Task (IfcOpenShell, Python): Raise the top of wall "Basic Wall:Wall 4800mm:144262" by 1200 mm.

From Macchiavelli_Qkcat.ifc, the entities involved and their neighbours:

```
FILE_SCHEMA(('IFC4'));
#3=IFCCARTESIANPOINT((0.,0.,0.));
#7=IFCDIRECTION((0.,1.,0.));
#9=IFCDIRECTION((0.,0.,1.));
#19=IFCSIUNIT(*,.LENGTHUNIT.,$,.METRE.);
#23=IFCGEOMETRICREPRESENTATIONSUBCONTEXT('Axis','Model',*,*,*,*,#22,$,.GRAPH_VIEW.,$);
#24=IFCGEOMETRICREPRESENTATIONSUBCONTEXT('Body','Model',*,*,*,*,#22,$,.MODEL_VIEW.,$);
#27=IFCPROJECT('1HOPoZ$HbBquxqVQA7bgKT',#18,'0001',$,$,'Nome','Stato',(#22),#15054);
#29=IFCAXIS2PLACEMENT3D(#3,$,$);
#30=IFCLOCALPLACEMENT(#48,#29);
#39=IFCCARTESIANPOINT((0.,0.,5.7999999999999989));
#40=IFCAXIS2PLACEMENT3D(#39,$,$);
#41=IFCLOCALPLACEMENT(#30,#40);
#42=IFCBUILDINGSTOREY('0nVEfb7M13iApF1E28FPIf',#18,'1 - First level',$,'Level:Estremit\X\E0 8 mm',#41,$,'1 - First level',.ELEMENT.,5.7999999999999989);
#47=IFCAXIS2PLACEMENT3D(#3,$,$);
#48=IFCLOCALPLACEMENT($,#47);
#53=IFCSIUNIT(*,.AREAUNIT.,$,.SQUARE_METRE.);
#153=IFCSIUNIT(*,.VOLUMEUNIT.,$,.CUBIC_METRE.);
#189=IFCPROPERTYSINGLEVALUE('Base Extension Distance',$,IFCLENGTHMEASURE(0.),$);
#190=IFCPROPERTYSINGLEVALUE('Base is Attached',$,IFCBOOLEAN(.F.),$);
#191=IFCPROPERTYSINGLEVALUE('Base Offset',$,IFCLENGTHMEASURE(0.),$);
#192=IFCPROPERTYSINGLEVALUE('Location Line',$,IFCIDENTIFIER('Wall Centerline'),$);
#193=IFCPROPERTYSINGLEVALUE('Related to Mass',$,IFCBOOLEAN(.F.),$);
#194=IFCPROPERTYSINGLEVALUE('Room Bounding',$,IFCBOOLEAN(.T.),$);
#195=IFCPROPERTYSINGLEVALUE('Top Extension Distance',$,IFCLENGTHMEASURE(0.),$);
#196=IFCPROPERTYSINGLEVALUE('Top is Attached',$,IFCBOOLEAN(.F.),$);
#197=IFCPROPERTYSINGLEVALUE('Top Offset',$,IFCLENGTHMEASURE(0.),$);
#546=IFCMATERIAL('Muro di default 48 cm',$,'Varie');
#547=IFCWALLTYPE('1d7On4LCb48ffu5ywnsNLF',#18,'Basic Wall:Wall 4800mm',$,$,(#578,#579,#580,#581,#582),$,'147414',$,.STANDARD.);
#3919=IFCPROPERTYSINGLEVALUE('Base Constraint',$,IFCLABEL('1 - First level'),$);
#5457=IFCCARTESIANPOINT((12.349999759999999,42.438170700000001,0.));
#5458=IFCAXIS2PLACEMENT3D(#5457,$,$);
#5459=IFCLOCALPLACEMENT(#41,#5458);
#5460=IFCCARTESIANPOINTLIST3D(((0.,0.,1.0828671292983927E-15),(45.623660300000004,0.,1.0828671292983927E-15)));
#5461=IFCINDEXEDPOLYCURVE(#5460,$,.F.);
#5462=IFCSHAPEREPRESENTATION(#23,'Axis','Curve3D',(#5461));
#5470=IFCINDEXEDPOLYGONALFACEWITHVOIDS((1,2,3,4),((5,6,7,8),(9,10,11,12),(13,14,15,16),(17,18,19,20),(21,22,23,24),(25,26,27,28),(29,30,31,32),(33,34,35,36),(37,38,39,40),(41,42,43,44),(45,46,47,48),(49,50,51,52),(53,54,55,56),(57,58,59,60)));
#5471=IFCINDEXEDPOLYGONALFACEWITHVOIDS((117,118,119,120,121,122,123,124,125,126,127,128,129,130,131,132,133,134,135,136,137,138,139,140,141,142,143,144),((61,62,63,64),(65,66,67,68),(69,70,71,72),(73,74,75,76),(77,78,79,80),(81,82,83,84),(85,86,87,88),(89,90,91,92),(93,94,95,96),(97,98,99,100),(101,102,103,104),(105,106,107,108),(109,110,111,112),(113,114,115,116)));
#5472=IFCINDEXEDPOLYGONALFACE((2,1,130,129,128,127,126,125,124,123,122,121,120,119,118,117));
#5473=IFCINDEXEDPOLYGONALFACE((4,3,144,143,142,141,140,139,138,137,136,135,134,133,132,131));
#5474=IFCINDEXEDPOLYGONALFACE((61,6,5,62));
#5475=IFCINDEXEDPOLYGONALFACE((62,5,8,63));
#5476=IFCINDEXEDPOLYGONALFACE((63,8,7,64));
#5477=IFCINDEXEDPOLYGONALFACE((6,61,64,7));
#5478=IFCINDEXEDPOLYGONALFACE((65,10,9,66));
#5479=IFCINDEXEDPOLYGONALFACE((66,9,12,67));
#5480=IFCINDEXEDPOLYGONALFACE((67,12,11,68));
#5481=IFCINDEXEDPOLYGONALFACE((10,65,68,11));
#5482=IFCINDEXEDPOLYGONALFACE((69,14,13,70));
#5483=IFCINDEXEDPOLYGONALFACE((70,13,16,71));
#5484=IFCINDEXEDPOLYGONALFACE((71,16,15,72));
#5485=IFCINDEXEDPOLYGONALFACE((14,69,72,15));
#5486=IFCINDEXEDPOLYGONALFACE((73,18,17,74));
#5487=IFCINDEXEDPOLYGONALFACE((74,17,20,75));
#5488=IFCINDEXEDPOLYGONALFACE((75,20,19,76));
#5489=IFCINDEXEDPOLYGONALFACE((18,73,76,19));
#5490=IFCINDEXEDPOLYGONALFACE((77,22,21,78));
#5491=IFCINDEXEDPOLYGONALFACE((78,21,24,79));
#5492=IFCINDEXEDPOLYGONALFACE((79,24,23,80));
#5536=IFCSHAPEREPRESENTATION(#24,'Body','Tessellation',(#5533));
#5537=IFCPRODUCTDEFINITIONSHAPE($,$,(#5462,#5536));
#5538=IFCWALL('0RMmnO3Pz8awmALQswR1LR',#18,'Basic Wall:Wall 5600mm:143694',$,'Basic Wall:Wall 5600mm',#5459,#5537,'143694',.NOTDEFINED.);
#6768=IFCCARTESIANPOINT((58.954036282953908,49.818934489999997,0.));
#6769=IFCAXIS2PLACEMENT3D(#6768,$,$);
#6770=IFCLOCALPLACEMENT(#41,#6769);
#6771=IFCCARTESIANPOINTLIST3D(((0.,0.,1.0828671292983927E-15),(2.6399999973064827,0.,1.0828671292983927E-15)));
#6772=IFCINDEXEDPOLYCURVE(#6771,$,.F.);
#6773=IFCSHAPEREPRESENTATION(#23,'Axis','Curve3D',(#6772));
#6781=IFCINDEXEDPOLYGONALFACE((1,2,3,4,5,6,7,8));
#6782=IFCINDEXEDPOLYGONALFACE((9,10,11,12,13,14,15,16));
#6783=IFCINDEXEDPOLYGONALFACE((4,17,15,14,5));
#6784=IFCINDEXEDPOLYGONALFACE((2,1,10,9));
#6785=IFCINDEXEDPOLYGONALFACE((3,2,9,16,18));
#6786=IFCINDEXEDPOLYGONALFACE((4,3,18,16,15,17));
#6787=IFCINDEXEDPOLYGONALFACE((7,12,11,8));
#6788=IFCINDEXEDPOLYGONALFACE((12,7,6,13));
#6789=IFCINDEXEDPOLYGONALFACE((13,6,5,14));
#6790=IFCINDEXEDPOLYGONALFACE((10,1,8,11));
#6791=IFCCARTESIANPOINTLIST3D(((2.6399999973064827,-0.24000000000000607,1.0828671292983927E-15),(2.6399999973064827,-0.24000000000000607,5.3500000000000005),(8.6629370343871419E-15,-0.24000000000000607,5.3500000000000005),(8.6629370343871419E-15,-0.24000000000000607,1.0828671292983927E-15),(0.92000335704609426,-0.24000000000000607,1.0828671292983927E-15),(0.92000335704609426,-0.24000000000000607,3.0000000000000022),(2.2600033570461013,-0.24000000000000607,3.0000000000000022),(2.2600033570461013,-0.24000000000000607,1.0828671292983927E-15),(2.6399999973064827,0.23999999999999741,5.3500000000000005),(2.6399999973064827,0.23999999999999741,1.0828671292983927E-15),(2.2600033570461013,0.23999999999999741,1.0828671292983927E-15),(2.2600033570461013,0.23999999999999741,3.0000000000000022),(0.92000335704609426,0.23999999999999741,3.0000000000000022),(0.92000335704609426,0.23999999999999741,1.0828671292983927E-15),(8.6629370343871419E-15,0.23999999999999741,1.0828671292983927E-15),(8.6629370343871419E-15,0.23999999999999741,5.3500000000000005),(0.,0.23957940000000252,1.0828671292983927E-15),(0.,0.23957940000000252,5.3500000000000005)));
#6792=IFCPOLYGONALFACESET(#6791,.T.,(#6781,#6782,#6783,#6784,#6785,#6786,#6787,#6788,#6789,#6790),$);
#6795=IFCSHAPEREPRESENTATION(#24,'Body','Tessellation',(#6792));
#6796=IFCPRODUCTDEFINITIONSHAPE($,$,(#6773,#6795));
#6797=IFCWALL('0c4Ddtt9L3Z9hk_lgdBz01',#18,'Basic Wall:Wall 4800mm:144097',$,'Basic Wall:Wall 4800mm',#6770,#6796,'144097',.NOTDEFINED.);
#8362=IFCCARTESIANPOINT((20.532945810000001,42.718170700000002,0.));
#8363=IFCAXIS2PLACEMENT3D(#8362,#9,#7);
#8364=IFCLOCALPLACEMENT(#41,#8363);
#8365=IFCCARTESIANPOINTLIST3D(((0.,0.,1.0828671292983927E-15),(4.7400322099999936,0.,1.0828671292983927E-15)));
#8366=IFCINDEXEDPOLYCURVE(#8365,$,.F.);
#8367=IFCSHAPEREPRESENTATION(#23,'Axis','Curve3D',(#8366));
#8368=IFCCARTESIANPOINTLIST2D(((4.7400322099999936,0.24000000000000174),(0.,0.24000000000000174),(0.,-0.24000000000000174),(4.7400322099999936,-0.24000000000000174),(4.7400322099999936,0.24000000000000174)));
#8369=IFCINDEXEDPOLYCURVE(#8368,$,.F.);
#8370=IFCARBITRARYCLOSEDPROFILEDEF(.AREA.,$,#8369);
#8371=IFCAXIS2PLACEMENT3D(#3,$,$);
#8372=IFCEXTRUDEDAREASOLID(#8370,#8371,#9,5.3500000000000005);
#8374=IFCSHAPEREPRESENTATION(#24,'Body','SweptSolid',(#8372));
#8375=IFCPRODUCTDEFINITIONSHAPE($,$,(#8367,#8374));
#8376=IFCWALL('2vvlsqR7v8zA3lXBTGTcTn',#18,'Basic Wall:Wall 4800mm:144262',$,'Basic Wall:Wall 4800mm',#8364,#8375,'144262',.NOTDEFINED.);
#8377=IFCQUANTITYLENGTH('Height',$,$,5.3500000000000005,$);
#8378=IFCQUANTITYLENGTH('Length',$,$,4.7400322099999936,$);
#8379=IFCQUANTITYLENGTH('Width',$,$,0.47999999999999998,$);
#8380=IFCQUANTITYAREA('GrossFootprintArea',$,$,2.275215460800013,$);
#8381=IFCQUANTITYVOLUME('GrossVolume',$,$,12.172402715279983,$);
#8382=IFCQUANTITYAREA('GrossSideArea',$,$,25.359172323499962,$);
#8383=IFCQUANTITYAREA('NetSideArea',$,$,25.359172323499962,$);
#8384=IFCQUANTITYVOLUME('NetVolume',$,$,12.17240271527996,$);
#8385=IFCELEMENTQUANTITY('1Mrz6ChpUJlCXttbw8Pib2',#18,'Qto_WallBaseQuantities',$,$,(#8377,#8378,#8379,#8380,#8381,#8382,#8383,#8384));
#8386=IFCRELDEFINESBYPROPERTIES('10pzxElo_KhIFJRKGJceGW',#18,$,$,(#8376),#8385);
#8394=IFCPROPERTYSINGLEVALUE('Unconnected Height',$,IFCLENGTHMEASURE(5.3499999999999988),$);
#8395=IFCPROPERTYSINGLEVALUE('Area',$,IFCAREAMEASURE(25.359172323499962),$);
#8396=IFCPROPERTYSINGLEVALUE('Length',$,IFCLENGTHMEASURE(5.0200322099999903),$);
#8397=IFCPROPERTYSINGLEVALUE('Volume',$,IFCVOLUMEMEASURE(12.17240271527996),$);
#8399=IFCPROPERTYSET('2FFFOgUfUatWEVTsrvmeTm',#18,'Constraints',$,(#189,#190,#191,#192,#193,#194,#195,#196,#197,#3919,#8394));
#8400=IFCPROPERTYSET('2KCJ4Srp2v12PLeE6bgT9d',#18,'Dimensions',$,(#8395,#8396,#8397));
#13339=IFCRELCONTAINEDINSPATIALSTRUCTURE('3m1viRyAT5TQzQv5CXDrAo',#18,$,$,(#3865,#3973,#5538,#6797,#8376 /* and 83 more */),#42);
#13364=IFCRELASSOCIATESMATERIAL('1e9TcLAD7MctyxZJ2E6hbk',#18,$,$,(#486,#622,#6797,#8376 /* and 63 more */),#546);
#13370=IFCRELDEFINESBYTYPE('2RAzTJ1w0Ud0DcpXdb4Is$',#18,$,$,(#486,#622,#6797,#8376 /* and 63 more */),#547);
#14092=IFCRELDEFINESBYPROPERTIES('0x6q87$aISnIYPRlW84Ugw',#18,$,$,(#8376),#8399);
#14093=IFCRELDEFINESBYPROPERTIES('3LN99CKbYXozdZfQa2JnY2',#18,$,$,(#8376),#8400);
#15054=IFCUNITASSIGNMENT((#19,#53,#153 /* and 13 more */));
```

```python
import ifcopenshell
import ifcopenshell.api.pset
import ifcopenshell.geom
import ifcopenshell.util.element
import ifcopenshell.util.representation
import ifcopenshell.util.shape
import ifcopenshell.util.unit

model = ifcopenshell.open("Macchiavelli_Qkcat.ifc")
unit_scale = ifcopenshell.util.unit.calculate_unit_scale(model)
area_scale = ifcopenshell.util.unit.calculate_unit_scale(model, "AREAUNIT")
volume_scale = ifcopenshell.util.unit.calculate_unit_scale(model, "VOLUMEUNIT")
settings = ifcopenshell.geom.settings()


def volume(element):
    """Net volume in cubic metres, openings subtracted."""
    shape = ifcopenshell.geom.create_shape(settings, element)
    return ifcopenshell.util.shape.get_volume(shape.geometry)


wall = model.by_guid("2vvlsqR7v8zA3lXBTGTcTn")
before = volume(wall)

body = ifcopenshell.util.representation.get_representation(wall, "Model", "Body")
solid = body.Items[0]
old_height = solid.Depth
solid.Depth += 1.2
after = volume(wall)
thickness = 0.48  # wall thickness in metres

# Update the stored height, areas and volumes.
qto = model.by_id(ifcopenshell.util.element.get_pset(wall, "Qto_WallBaseQuantities", should_inherit=False)["id"])
ifcopenshell.api.pset.edit_qto(model, qto=qto, properties={
    "Height": solid.Depth,
    "GrossVolume": ifcopenshell.util.element.get_pset(wall, "Qto_WallBaseQuantities", "GrossVolume") * solid.Depth / old_height,
    "GrossSideArea": ifcopenshell.util.element.get_pset(wall, "Qto_WallBaseQuantities", "GrossSideArea") * solid.Depth / old_height,
    "NetSideArea": after / thickness / area_scale,
    "NetVolume": after / volume_scale,
})
pset = model.by_id(ifcopenshell.util.element.get_pset(wall, "Constraints", should_inherit=False)["id"])
ifcopenshell.api.pset.edit_pset(model, pset=pset, properties={
    "Unconnected Height": model.create_entity("IfcLengthMeasure", solid.Depth),
})
pset = model.by_id(ifcopenshell.util.element.get_pset(wall, "Dimensions", should_inherit=False)["id"])
ifcopenshell.api.pset.edit_pset(model, pset=pset, properties={
    "Area": model.create_entity("IfcAreaMeasure", after / thickness / area_scale),
    "Volume": model.create_entity("IfcVolumeMeasure", after / volume_scale),
})

print(f"height {old_height:g} -> {solid.Depth:g}, volume {before:.3f} -> {after:.3f} m3")

model.write("Macchiavelli_Qkcat_edited.ifc")
```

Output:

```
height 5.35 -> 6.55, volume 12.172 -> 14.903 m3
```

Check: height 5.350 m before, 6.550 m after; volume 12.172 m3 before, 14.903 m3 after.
